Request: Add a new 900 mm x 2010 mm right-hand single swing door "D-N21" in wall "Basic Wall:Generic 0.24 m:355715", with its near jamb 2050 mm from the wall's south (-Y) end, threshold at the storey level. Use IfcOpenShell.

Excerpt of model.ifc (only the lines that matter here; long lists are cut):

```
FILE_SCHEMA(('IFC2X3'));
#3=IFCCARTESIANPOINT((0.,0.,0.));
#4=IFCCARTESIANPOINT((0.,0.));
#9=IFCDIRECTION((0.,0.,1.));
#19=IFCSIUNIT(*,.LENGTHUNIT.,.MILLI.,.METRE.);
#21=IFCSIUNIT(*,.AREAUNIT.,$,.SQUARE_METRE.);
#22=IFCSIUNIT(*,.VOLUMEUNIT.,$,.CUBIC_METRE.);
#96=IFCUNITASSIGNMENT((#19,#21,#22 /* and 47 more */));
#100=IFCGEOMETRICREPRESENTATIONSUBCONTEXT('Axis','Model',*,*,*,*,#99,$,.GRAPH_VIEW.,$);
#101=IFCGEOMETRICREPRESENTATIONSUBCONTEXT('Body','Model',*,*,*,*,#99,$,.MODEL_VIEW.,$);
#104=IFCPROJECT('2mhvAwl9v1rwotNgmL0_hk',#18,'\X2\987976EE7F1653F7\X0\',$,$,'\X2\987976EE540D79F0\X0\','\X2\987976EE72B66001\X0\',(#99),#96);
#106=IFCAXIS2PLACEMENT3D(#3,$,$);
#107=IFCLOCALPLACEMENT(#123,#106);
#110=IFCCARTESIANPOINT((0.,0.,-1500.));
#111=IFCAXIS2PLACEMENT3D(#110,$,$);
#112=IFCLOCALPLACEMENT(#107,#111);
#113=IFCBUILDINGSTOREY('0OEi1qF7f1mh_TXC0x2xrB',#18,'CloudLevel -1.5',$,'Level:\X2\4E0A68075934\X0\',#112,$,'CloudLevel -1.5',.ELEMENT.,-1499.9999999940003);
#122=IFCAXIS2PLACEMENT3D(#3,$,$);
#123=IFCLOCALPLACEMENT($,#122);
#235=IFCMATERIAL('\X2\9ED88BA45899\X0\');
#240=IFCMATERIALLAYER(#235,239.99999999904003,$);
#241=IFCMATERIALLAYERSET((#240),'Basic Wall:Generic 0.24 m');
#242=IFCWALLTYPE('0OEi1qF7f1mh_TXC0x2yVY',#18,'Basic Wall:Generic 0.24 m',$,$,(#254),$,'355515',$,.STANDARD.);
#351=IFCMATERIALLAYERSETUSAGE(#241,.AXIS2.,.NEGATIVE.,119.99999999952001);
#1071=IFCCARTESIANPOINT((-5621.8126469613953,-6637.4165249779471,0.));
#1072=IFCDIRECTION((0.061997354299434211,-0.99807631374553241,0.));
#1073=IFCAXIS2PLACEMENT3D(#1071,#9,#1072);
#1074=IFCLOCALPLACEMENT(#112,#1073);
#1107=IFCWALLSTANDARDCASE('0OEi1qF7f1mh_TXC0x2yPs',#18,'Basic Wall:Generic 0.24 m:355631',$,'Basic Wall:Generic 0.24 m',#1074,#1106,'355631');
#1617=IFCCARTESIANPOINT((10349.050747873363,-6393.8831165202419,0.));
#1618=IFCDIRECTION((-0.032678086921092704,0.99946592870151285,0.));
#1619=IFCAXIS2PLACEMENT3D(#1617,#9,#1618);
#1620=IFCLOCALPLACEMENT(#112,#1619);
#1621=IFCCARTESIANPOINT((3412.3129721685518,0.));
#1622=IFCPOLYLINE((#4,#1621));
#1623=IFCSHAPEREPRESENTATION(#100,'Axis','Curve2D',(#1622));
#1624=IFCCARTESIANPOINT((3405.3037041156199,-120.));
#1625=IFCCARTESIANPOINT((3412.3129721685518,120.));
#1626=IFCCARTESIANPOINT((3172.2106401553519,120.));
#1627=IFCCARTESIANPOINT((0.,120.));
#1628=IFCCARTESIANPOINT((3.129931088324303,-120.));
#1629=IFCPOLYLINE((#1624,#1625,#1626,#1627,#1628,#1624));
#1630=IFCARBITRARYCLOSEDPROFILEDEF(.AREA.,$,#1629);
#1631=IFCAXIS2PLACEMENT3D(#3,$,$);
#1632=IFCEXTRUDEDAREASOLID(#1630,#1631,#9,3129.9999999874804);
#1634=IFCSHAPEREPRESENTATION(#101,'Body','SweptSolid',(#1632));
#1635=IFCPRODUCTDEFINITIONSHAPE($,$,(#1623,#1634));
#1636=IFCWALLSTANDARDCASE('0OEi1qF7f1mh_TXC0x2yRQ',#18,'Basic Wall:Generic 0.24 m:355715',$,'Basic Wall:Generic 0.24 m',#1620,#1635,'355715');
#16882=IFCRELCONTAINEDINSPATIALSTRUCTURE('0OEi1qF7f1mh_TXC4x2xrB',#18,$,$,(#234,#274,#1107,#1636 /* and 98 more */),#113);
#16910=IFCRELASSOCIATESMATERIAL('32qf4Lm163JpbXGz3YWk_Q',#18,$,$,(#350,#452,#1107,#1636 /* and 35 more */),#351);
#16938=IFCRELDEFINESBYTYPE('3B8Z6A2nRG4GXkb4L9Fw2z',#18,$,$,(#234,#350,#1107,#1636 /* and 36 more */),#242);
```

```python
import numpy as np
import ifcopenshell
import ifcopenshell.api.feature
import ifcopenshell.api.geometry
import ifcopenshell.api.root
import ifcopenshell.api.spatial
import ifcopenshell.api.type
import ifcopenshell.geom
import ifcopenshell.util.element
import ifcopenshell.util.placement
import ifcopenshell.util.representation
import ifcopenshell.util.shape
import ifcopenshell.util.unit

model = ifcopenshell.open("model.ifc")
unit_scale = ifcopenshell.util.unit.calculate_unit_scale(model)
settings = ifcopenshell.geom.settings()


def volume(element):
    """Net volume in cubic metres, openings subtracted."""
    shape = ifcopenshell.geom.create_shape(settings, element)
    return ifcopenshell.util.shape.get_volume(shape.geometry)


wall = model.by_guid("0OEi1qF7f1mh_TXC0x2yRQ")
storey = ifcopenshell.util.element.get_container(wall, ifc_class="IfcBuildingStorey")
context = ifcopenshell.util.representation.get_context(model, "Model", "Body", "MODEL_VIEW")
before = volume(wall)

width, height, from_end, sill = 0.9, 2.01, 2.05, 0.0  # metres

# The wall runs along its own X axis, and the end named is its -X end.
wall_shape = ifcopenshell.geom.create_shape(settings, wall)
x, y, z = ifcopenshell.util.shape.get_vertices(wall_shape.geometry).T
start = x.min() + from_end
face, thickness = float(y.min()), float(y.max() - y.min())
wall_matrix = ifcopenshell.util.placement.get_local_placement(wall.ObjectPlacement)
level = ifcopenshell.util.placement.get_local_placement(storey.ObjectPlacement)[2, 3]


def in_wall(x, y):
    """Placement at x, y metres in the wall's axes, at sill height."""
    matrix = wall_matrix.copy()
    matrix[:, 3] = wall_matrix @ np.array([x / unit_scale, y / unit_scale, 0.0, 1.0])
    matrix[2, 3] = level + sill / unit_scale
    return matrix


# Opening: a box that overshoots both wall faces by 50 mm.
opening = ifcopenshell.api.root.create_entity(model, ifc_class="IfcOpeningElement")
box = ifcopenshell.api.geometry.add_wall_representation(
    model, context=context, length=width, height=height, thickness=thickness + 0.1
)
ifcopenshell.api.geometry.assign_representation(model, product=opening, representation=box)
ifcopenshell.api.geometry.edit_object_placement(model, product=opening, matrix=in_wall(start, face - 0.05), is_si=False)
ifcopenshell.api.feature.add_feature(model, feature=opening, element=wall)

door = ifcopenshell.api.root.create_entity(model, ifc_class="IfcDoor", name="D-N21")
door.OverallWidth, door.OverallHeight = width / unit_scale, height / unit_scale
body = ifcopenshell.api.geometry.add_door_representation(
    model,
    context=context,
    overall_width=door.OverallWidth,
    overall_height=door.OverallHeight,
    operation_type="SINGLE_SWING_RIGHT",
    lining_properties={"LiningDepth": thickness / unit_scale, "ThresholdDepth": thickness / unit_scale},
)
ifcopenshell.api.geometry.assign_representation(model, product=door, representation=body)
ifcopenshell.api.spatial.assign_container(model, products=[door], relating_structure=storey)
fills = ifcopenshell.api.feature.add_filling(model, opening=opening, element=door)
fills.OwnerHistory = door.OwnerHistory  # required in IFC2X3

# IFC2X3 keeps the operation on the door style.
style = ifcopenshell.api.root.create_entity(model, ifc_class="IfcDoorStyle", name="D-N21")
style.OperationType, style.ConstructionType = "SINGLE_SWING_RIGHT", "NOTDEFINED"
style.ParameterTakesPrecedence = style.Sizeable = False
ifcopenshell.api.type.assign_type(model, related_objects=[door], relating_type=style)

# The lining spans the wall, so the door starts at the wall face.
ifcopenshell.api.geometry.edit_object_placement(model, product=door, matrix=in_wall(start, face), is_si=False)

after = volume(wall)

print(f"wall volume {before:.3f} -> {after:.3f} m3")

model.write("model_rev.ifc")
```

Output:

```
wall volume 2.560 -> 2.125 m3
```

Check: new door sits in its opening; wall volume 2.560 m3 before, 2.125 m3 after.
